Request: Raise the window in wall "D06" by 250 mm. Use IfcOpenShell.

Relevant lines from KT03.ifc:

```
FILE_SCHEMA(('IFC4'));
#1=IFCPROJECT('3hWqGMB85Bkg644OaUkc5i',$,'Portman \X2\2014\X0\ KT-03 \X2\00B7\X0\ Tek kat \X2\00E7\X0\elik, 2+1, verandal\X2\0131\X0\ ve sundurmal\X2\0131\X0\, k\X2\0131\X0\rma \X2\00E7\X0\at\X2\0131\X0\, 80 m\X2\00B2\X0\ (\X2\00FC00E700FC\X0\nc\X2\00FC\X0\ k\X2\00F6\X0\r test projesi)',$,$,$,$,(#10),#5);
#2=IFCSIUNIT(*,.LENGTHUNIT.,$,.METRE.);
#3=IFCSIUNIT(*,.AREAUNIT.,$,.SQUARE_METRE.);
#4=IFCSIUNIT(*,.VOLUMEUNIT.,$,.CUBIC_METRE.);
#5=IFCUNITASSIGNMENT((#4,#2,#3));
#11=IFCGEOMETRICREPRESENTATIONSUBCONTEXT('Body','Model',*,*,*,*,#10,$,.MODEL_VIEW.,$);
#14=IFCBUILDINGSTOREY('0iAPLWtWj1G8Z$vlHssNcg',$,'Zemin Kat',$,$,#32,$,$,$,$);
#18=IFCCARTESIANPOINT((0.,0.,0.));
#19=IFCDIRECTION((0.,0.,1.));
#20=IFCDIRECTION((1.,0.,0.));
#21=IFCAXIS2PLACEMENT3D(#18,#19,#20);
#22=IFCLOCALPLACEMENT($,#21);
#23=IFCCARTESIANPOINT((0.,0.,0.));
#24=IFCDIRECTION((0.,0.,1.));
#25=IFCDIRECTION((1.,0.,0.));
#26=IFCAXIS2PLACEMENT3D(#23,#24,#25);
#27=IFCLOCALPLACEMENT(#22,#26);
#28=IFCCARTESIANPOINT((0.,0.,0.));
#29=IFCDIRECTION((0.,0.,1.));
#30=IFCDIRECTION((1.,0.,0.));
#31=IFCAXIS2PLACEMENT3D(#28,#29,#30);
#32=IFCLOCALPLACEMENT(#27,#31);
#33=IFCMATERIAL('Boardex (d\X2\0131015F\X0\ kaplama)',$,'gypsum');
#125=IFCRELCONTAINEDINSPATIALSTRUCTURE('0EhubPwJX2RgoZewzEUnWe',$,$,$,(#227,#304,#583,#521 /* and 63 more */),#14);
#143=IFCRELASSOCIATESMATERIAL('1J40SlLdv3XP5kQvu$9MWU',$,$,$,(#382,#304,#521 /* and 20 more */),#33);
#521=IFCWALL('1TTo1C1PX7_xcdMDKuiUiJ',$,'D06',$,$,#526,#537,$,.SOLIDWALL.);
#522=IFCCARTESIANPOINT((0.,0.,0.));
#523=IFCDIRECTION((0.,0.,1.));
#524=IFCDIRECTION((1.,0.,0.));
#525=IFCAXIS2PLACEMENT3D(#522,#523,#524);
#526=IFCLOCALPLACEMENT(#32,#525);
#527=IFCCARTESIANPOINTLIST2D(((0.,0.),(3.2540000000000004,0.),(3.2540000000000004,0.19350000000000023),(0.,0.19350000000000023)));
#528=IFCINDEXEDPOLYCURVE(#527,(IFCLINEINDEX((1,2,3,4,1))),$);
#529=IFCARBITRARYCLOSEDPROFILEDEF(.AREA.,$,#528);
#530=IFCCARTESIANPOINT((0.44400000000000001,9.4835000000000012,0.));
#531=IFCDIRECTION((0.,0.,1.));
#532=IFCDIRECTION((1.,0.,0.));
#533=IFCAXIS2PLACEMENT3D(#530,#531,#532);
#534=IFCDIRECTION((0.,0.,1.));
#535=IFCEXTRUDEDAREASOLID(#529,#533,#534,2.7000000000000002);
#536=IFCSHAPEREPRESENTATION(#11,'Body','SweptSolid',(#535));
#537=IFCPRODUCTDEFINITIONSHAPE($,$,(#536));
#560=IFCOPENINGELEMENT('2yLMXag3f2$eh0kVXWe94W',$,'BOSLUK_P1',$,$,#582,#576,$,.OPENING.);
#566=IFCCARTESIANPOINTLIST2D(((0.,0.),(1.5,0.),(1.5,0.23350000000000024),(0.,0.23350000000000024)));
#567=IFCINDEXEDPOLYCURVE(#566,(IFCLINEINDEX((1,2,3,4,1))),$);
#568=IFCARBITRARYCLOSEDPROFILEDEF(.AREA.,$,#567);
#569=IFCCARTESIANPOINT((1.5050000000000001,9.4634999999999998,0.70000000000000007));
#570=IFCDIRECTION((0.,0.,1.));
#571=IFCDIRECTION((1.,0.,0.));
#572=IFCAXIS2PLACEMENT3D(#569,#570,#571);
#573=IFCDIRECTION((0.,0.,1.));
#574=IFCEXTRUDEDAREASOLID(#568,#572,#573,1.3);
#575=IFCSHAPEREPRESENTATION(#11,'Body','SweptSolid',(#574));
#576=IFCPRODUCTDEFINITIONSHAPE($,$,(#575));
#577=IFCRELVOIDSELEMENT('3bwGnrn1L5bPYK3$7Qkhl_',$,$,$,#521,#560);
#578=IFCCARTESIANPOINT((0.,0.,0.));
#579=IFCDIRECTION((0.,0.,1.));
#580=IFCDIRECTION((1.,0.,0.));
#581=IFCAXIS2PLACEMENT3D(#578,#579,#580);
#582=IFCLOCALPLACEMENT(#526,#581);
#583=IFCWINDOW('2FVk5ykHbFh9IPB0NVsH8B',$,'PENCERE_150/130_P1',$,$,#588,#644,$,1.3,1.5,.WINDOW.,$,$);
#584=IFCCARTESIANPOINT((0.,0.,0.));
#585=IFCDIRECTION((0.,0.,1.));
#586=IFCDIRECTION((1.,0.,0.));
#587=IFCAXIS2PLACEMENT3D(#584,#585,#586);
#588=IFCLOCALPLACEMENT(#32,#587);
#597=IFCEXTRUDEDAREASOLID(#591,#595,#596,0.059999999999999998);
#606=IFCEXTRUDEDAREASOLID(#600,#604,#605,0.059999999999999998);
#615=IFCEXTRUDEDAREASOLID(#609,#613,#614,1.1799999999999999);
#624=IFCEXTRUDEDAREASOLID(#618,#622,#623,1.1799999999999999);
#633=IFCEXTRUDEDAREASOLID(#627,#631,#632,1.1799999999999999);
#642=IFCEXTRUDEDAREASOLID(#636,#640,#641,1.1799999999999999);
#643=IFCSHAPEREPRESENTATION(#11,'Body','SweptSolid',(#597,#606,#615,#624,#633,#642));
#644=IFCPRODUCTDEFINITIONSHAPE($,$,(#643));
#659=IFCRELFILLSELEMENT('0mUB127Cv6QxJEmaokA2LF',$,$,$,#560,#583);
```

```python
import numpy as np
import ifcopenshell
import ifcopenshell.api.geometry
import ifcopenshell.util.placement
import ifcopenshell.util.unit

model = ifcopenshell.open("KT03.ifc")
unit_scale = ifcopenshell.util.unit.calculate_unit_scale(model)

window = model.by_guid("2FVk5ykHbFh9IPB0NVsH8B")
opening = window.FillsVoids[0].RelatingOpeningElement
dz = 0.25

shift = np.array([0.0, 0.0, dz])
# The window is not placed relative to its opening, so move both.
for product in (opening, window):
    matrix = ifcopenshell.util.placement.get_local_placement(product.ObjectPlacement)
    matrix[:3, 3] += shift
    ifcopenshell.api.geometry.edit_object_placement(model, product=product, matrix=matrix, is_si=False)

print(f"moved by {dz * unit_scale:+.3f} m")

model.write("KT03_rev.ifc")
```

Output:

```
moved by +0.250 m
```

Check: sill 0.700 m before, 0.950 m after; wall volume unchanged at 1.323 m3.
